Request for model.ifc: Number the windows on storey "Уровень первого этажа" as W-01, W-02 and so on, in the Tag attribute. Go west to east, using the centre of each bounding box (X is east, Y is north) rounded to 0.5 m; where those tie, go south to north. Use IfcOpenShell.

First a look at what the model holds.

```python
import ifcopenshell
import ifcopenshell.util.element
import ifcopenshell.util.placement

model = ifcopenshell.open("model.ifc")
print(model.schema)
storey = next(s for s in model.by_type("IfcBuildingStorey") if s.Name == "Уровень первого этажа")
windows = [e for e in ifcopenshell.util.element.get_decomposition(storey) if e.is_a("IfcWindow")]
for e in sorted(windows, key=lambda e: e.id()):
    origin = ifcopenshell.util.placement.get_local_placement(e.ObjectPlacement)[:3, 3]
    print(e.id(), e.Tag, e.Name, origin.round(2) + 0.0, sep=" | ")
```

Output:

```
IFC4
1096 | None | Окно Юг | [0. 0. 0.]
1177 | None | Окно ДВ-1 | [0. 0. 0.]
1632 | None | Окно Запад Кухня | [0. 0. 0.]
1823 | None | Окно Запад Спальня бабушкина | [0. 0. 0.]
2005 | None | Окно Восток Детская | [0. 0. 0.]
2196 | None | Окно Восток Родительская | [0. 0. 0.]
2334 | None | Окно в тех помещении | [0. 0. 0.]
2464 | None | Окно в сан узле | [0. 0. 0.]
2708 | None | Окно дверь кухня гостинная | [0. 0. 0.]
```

```python
import ifcopenshell
import ifcopenshell.geom
import ifcopenshell.util.element
import ifcopenshell.util.shape

model = ifcopenshell.open("model.ifc")
settings = ifcopenshell.geom.settings()
settings.set("use-world-coords", True)


def centre(element):
    shape = ifcopenshell.geom.create_shape(settings, element)
    return ifcopenshell.util.shape.get_bbox_centroid(shape.geometry)


storey = next(s for s in model.by_type("IfcBuildingStorey") if s.Name == "Уровень первого этажа")
windows = [e for e in ifcopenshell.util.element.get_decomposition(storey) if e.is_a("IfcWindow")]

# Insertion points can sit at a corner or the storey origin, so sort by the geometry (in metres).
centres = {e: centre(e) for e in windows}
windows.sort(key=lambda e: (round(centres[e][0] / 0.5), centres[e][1]))

for i, e in enumerate(windows, start=1):
    number = f"W-{i:02d}"
    e.Tag = number
    print(e.id(), number)

model.write("model_updated.ifc")
```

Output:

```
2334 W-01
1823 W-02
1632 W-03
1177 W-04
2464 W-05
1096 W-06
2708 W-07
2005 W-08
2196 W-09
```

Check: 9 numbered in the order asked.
